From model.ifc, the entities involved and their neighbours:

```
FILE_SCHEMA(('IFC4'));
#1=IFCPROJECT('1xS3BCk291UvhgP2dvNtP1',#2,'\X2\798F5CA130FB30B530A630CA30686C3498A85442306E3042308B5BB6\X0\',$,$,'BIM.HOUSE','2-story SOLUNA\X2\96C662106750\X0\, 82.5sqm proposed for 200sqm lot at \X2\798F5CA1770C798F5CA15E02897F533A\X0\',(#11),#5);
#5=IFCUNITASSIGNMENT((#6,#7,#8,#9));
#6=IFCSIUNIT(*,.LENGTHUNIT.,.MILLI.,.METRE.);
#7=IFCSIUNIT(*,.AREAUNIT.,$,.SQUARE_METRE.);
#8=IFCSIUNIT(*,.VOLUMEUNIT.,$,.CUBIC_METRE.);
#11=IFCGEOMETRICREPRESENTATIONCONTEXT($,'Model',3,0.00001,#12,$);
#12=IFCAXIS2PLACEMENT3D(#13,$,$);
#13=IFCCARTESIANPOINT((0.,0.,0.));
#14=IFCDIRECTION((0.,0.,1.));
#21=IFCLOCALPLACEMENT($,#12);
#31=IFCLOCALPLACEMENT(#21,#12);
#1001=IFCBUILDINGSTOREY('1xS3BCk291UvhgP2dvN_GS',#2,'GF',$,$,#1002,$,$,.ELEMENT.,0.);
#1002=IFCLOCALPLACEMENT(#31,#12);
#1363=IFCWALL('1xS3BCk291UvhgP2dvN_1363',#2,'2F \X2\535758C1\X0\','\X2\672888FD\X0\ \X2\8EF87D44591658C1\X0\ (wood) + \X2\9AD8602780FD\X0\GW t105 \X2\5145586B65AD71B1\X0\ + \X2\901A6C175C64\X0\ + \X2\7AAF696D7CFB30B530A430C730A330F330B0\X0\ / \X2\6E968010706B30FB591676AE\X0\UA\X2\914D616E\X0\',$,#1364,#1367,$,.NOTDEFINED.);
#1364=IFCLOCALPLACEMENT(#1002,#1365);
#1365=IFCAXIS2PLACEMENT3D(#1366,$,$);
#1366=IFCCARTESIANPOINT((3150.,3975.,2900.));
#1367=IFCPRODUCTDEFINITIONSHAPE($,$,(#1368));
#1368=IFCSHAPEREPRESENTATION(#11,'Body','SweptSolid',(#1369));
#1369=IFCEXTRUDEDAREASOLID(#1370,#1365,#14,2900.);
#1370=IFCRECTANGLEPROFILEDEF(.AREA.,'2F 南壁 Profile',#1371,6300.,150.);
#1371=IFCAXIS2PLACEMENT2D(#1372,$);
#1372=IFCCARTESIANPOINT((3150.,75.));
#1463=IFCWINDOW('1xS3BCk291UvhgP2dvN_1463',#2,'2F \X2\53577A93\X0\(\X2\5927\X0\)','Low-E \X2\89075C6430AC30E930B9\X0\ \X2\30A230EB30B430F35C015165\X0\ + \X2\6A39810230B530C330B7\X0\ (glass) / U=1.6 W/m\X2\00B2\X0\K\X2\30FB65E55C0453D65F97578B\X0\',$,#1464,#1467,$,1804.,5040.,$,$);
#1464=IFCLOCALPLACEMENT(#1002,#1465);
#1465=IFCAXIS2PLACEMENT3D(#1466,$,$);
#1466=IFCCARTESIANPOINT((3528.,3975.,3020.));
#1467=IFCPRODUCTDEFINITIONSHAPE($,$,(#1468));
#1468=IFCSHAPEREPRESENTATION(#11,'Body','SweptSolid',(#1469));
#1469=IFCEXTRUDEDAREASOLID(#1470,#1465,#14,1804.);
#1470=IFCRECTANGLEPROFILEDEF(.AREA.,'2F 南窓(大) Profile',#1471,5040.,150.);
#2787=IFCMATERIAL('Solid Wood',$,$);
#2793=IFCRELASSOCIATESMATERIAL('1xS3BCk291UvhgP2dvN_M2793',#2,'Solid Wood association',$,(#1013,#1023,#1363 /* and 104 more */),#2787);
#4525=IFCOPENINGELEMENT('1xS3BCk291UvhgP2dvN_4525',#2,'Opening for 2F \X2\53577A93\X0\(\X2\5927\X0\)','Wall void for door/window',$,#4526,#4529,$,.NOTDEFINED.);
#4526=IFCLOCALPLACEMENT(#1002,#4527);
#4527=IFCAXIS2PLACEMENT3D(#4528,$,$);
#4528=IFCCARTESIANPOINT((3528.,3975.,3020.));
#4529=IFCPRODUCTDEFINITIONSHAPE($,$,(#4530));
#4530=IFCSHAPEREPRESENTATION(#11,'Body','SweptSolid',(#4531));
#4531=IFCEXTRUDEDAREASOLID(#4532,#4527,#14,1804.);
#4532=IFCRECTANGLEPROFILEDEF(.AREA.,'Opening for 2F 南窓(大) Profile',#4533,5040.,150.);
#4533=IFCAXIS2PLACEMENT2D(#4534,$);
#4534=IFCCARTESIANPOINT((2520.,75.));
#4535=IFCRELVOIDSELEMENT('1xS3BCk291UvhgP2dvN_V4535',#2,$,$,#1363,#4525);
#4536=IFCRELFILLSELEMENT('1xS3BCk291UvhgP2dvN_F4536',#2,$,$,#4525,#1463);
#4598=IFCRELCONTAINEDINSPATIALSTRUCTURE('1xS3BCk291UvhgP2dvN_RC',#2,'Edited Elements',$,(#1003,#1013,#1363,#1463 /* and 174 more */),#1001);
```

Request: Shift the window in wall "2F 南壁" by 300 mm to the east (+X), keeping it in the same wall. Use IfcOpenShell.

```python
import ifcopenshell
import ifcopenshell.api.geometry
import ifcopenshell.util.placement
import ifcopenshell.util.unit

model = ifcopenshell.open("model.ifc")
unit_scale = ifcopenshell.util.unit.calculate_unit_scale(model)

window = model.by_guid("1xS3BCk291UvhgP2dvN_1463")
opening = window.FillsVoids[0].RelatingOpeningElement
wall = opening.VoidsElements[0].RelatingBuildingElement

wall_matrix = ifcopenshell.util.placement.get_local_placement(wall.ObjectPlacement)
shift = wall_matrix[:3, 0] * 0.3 / unit_scale
before = ifcopenshell.util.placement.get_local_placement(window.ObjectPlacement)[:3, 3].copy()

# The window is not placed relative to its opening, so move both.
for product in (opening, window):
    matrix = ifcopenshell.util.placement.get_local_placement(product.ObjectPlacement)
    matrix[:3, 3] += shift
    ifcopenshell.api.geometry.edit_object_placement(model, product=product, matrix=matrix, is_si=False)

after = ifcopenshell.util.placement.get_local_placement(window.ObjectPlacement)[:3, 3]
print("window moved by", (after - before).round(3) + 0.0)

model.write("model-out.ifc")
```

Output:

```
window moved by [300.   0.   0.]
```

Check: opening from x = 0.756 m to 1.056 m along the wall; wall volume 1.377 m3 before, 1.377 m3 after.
